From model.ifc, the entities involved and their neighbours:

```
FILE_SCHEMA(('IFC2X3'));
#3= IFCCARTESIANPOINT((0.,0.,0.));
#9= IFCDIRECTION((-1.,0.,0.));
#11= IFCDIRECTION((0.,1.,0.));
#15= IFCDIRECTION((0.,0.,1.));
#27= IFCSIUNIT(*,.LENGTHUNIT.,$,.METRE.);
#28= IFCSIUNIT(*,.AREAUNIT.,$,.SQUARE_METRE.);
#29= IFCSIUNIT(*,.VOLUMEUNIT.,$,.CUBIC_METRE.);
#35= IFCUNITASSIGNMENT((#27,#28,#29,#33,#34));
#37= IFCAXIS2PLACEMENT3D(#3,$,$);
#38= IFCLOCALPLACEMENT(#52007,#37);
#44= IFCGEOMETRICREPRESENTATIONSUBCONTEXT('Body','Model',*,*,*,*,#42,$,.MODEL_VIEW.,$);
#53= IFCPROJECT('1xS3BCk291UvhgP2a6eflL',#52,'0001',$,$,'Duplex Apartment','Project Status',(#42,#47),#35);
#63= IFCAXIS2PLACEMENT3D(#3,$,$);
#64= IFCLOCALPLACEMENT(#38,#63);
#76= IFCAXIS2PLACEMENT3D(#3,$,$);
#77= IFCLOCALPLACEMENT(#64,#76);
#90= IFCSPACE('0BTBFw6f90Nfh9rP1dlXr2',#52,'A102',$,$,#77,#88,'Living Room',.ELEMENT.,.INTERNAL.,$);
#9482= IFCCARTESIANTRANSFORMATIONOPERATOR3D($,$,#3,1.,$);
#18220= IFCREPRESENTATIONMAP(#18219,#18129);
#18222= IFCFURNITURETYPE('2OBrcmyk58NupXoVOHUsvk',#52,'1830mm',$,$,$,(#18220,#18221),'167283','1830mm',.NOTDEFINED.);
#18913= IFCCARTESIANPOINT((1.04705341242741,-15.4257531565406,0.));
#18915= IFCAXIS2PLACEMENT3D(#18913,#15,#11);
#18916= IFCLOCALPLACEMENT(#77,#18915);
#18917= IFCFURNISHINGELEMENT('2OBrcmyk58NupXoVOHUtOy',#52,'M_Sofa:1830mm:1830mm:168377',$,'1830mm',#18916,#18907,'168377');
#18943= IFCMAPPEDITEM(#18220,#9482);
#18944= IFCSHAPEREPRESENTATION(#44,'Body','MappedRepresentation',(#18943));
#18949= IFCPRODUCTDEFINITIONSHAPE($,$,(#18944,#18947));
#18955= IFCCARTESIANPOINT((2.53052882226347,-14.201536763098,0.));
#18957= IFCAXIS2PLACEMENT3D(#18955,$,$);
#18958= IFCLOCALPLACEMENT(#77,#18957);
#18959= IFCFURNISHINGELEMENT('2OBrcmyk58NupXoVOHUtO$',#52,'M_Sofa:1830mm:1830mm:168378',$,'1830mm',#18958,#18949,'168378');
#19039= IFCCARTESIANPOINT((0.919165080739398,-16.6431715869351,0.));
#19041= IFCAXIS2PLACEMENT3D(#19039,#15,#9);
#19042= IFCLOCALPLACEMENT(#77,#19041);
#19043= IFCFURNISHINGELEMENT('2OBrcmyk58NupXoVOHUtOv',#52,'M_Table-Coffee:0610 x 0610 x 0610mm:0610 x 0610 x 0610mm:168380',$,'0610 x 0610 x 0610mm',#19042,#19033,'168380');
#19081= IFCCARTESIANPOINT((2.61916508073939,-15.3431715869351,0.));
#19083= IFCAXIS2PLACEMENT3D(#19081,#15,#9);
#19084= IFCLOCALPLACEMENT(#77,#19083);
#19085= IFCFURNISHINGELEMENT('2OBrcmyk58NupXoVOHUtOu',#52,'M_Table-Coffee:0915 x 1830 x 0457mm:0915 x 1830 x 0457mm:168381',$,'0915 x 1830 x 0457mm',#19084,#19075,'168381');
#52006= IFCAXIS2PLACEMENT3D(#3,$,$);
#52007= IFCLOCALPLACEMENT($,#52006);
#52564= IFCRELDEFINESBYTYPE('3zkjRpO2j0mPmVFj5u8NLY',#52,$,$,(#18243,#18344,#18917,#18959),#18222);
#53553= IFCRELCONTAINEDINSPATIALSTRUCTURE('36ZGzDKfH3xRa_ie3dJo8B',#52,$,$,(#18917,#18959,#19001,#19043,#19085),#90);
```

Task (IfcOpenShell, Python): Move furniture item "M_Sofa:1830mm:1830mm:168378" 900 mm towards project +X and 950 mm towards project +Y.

```python
import ifcopenshell
import ifcopenshell.api.geometry
import ifcopenshell.util.placement

model = ifcopenshell.open("model.ifc")

item = model.by_id(18959)
matrix = ifcopenshell.util.placement.get_local_placement(item.ObjectPlacement)
matrix[0, 3] += 0.9
matrix[1, 3] += 0.95
ifcopenshell.api.geometry.edit_object_placement(model, product=item, matrix=matrix, is_si=False)

print(ifcopenshell.util.placement.get_local_placement(item.ObjectPlacement).round(3) + 0.0)

model.write("model_v2.ifc")
```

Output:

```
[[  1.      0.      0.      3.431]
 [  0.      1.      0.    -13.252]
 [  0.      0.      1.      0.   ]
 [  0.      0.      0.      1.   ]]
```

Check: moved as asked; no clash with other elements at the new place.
